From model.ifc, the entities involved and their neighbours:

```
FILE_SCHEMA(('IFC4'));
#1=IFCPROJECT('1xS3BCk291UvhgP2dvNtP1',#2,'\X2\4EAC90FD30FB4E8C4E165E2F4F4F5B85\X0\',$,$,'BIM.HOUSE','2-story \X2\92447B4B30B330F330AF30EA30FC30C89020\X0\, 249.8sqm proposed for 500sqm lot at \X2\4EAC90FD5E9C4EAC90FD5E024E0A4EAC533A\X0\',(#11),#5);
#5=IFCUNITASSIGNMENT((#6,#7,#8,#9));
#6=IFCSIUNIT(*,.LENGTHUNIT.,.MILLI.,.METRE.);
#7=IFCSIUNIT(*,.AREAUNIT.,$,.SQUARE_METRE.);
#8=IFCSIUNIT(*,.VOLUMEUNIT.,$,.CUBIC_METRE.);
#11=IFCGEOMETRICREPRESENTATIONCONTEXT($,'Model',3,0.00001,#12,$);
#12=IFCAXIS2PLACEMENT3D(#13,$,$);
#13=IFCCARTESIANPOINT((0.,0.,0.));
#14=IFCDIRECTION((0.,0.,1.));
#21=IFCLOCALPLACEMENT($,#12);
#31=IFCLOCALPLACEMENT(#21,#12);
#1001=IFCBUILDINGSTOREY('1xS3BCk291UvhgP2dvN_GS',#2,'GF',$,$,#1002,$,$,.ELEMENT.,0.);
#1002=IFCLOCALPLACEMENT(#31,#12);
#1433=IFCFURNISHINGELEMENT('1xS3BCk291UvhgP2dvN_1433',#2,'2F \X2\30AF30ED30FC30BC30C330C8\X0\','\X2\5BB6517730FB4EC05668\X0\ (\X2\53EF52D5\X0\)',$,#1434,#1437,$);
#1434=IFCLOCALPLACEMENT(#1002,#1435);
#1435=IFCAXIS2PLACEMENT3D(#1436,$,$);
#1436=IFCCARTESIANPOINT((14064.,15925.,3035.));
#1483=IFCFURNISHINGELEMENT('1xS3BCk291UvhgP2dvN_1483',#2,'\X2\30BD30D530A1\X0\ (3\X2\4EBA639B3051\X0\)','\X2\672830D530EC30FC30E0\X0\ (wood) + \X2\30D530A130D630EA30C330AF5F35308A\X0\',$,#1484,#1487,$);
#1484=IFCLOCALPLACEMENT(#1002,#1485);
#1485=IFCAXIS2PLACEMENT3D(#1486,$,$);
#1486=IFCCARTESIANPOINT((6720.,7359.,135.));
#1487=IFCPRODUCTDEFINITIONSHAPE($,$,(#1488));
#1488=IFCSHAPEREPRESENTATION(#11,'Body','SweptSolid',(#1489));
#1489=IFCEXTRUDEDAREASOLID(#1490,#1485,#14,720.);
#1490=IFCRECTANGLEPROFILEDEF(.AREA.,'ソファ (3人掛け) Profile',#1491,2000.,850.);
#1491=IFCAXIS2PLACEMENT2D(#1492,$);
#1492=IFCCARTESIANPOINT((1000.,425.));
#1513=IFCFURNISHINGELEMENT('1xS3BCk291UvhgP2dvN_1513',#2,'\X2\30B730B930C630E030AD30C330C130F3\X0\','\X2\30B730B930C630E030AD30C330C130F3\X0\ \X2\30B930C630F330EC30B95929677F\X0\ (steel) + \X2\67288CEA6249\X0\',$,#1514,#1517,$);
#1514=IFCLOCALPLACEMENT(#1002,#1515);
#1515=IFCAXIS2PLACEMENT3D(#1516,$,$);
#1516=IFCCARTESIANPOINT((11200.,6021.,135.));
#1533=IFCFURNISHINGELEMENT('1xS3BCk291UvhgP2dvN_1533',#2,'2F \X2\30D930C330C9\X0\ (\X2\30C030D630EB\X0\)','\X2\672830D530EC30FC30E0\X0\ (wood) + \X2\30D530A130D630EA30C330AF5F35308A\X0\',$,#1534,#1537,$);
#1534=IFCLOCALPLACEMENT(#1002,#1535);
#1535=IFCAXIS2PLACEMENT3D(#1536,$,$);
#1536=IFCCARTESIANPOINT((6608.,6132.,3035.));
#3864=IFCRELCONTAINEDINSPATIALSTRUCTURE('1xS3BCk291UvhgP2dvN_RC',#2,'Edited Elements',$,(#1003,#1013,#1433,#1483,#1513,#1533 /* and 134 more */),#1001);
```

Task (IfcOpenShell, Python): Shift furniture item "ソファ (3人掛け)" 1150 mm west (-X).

```python
import ifcopenshell
import ifcopenshell.api.geometry
import ifcopenshell.util.placement

model = ifcopenshell.open("model.ifc")

item = model.by_guid("1xS3BCk291UvhgP2dvN_1483")
matrix = ifcopenshell.util.placement.get_local_placement(item.ObjectPlacement)
matrix[0, 3] -= 1150.0
ifcopenshell.api.geometry.edit_object_placement(model, product=item, matrix=matrix, is_si=False)

print(ifcopenshell.util.placement.get_local_placement(item.ObjectPlacement).round(3) + 0.0)

model.write("model_updated.ifc")
```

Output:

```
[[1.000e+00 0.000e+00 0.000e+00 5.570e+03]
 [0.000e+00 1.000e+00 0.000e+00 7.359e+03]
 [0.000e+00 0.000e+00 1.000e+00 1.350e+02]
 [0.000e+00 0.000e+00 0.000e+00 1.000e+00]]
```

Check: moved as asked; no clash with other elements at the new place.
